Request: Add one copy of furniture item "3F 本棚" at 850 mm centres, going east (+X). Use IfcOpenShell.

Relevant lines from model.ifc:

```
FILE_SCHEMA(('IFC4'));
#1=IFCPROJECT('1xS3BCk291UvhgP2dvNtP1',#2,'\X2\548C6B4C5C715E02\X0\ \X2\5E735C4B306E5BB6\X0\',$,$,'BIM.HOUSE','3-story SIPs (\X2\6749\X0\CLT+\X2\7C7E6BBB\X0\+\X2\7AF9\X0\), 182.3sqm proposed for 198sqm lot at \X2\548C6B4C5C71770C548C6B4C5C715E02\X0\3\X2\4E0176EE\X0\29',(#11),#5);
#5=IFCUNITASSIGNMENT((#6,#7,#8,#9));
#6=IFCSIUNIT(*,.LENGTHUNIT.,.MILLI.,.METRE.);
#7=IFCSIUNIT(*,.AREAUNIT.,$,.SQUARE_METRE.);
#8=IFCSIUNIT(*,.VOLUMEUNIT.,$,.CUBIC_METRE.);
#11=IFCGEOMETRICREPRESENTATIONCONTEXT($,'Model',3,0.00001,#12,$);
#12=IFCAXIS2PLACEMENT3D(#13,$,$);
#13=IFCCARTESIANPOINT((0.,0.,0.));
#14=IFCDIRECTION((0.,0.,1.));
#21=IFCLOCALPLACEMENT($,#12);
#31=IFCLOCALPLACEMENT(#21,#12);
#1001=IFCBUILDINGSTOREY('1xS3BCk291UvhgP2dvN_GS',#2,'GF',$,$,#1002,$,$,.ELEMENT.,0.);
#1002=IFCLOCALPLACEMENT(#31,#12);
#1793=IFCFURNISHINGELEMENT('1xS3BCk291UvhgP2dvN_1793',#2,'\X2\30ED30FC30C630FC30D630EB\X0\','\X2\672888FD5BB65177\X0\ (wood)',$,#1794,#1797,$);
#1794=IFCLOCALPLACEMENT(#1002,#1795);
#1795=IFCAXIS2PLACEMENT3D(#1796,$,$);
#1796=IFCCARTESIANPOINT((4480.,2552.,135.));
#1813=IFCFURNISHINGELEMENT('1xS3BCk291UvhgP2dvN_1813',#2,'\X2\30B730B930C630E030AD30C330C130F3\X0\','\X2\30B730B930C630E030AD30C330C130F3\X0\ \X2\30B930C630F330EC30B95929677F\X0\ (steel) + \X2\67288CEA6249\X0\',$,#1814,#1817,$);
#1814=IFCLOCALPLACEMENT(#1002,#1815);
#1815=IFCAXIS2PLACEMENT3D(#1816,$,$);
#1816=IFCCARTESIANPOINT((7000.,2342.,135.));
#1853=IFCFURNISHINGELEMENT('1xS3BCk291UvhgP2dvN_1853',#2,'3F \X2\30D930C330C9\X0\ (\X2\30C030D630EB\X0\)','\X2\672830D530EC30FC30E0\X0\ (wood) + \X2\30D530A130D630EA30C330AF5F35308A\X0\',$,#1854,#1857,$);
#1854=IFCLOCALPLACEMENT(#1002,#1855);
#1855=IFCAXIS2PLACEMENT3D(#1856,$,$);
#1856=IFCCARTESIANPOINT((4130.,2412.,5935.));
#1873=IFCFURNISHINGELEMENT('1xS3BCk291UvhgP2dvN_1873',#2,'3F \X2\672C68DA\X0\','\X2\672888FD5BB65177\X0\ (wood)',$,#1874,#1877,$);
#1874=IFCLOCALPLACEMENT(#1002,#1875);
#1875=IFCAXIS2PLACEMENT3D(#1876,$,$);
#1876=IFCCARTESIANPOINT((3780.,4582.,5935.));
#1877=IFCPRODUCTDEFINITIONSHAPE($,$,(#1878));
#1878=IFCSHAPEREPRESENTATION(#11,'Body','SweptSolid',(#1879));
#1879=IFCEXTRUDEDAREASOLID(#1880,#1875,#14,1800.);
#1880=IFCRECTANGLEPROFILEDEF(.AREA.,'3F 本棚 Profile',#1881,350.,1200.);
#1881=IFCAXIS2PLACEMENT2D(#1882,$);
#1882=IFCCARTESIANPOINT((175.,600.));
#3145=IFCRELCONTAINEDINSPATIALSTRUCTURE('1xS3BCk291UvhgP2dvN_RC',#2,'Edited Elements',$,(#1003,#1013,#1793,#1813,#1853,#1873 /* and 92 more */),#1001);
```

```python
import numpy as np
import ifcopenshell
import ifcopenshell.api.geometry
import ifcopenshell.api.root
import ifcopenshell.util.element
import ifcopenshell.util.placement

model = ifcopenshell.open("model.ifc")


def reuse_history(source, copy):
    """copy_class also copies each property set's owner history, people and application; keep the originals."""
    for rel in copy.IsDefinedBy:
        if rel.is_a("IfcRelDefinesByProperties") and (history := rel.RelatingPropertyDefinition.OwnerHistory):
            rel.RelatingPropertyDefinition.OwnerHistory = source.OwnerHistory
            ifcopenshell.util.element.remove_deep2(model, history)


source = model.by_id(1873)
base = ifcopenshell.util.placement.get_local_placement(source.ObjectPlacement)
step = np.array([1.0, 0.0, 0.0]) * 850.0

for i in range(1, 2):
    copy = ifcopenshell.api.root.copy_class(model, product=source)
    copy.Representation = ifcopenshell.util.element.copy_deep(
        model, source.Representation, exclude=["IfcGeometricRepresentationContext", "IfcRepresentationMap"]
    )
    reuse_history(source, copy)
    matrix = base.copy()
    matrix[:3, 3] += i * step
    print("added at", matrix[:3, 3].round(3) + 0.0)
    ifcopenshell.api.geometry.edit_object_placement(model, product=copy, matrix=matrix, is_si=False)

model.write("model_rev.ifc")
```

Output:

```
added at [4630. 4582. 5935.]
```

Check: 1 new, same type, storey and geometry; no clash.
